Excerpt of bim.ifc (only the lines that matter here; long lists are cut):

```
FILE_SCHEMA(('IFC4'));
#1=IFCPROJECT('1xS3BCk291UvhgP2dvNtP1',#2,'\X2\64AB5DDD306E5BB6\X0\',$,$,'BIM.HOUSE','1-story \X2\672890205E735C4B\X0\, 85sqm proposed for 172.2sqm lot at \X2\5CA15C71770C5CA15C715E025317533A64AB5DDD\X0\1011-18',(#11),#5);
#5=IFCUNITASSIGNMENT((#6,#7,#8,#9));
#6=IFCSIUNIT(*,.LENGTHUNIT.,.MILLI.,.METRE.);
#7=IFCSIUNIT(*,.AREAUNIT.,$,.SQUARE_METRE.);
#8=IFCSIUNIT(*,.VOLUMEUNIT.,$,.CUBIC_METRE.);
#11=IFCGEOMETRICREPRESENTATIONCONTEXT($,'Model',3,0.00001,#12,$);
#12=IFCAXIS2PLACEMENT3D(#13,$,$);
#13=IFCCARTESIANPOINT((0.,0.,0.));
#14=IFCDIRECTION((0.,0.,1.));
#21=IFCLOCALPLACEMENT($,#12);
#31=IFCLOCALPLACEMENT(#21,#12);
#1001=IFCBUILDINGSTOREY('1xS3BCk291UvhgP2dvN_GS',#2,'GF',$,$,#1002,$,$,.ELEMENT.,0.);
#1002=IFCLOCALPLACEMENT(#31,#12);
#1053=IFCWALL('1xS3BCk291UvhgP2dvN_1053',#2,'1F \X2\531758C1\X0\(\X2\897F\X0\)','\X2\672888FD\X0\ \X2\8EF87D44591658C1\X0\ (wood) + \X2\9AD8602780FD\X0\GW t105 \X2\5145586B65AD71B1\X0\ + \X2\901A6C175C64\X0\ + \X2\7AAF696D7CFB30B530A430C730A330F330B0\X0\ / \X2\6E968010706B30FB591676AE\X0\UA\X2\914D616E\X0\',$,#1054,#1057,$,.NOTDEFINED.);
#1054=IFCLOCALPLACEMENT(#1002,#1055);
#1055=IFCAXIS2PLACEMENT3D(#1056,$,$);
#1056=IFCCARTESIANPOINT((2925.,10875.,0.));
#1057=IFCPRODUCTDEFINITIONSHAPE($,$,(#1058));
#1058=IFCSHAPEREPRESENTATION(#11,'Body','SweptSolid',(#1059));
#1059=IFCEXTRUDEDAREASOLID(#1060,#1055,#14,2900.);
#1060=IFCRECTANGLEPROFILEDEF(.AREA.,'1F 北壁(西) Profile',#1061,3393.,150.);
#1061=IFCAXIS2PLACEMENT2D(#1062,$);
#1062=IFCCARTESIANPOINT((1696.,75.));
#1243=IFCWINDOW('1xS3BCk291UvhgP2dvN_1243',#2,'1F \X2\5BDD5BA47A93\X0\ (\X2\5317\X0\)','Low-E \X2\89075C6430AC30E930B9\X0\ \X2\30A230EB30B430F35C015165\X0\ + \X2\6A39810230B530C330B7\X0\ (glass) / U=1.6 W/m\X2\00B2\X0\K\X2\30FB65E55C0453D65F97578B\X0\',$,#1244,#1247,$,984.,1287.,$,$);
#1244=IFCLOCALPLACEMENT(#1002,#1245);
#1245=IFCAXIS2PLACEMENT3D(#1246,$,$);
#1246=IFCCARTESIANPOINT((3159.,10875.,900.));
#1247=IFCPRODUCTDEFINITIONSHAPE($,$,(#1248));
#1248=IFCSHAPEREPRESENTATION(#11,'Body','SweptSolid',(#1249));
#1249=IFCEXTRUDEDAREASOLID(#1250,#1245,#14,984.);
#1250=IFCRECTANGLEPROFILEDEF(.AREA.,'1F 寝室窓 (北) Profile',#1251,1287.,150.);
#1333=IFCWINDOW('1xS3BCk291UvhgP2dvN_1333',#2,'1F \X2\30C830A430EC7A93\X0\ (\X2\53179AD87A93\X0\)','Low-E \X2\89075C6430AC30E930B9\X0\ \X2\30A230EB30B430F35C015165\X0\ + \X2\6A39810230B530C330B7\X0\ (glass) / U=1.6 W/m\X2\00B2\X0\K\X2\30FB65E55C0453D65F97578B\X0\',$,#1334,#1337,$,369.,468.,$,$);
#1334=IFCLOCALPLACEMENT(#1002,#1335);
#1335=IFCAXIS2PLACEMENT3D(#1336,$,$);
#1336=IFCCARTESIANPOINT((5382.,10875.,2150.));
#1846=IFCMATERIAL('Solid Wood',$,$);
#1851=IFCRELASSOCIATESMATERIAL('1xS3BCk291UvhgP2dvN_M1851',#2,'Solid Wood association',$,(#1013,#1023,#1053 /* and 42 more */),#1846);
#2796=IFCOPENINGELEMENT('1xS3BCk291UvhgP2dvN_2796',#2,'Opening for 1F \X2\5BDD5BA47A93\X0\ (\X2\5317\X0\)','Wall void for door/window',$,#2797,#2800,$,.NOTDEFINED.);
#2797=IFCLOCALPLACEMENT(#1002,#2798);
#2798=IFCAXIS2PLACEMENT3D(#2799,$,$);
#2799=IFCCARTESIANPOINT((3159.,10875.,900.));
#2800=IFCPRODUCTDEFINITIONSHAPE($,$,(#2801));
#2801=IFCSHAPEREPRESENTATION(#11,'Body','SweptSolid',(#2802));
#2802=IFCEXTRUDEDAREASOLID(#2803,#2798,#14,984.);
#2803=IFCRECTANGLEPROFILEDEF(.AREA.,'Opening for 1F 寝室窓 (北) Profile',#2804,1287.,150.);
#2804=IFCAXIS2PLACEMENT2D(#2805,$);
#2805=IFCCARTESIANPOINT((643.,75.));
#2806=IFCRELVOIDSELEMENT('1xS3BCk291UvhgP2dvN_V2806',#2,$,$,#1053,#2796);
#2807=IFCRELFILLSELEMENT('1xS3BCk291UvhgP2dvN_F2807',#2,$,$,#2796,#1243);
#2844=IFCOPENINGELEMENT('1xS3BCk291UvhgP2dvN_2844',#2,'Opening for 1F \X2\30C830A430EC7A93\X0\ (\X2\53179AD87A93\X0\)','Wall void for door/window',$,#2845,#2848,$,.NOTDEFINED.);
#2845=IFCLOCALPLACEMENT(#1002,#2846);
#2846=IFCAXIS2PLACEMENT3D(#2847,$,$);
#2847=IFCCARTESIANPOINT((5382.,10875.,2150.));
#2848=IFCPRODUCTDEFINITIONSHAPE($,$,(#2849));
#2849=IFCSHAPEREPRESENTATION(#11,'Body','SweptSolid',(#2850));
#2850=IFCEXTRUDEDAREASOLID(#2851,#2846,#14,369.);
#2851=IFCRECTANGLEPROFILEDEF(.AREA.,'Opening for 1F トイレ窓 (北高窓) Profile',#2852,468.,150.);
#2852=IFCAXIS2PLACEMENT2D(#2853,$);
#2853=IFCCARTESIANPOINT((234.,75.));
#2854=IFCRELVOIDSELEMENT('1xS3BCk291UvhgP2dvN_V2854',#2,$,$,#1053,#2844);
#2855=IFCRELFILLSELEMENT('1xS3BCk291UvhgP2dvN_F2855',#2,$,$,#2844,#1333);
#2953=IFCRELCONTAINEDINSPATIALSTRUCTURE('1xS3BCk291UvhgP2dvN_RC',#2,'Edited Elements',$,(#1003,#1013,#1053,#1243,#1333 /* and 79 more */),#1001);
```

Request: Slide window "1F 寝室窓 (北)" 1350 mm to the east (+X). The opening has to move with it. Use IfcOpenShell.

```python
import ifcopenshell
import ifcopenshell.api.geometry
import ifcopenshell.util.placement
import ifcopenshell.util.unit

model = ifcopenshell.open("bim.ifc")
unit_scale = ifcopenshell.util.unit.calculate_unit_scale(model)

window = model.by_guid("1xS3BCk291UvhgP2dvN_1243")
opening = window.FillsVoids[0].RelatingOpeningElement
wall = opening.VoidsElements[0].RelatingBuildingElement

wall_matrix = ifcopenshell.util.placement.get_local_placement(wall.ObjectPlacement)
shift = wall_matrix[:3, 0] * 1.35 / unit_scale
before = ifcopenshell.util.placement.get_local_placement(window.ObjectPlacement)[:3, 3].copy()

# The window is not placed relative to its opening, so move both.
for product in (opening, window):
    matrix = ifcopenshell.util.placement.get_local_placement(product.ObjectPlacement)
    matrix[:3, 3] += shift
    ifcopenshell.api.geometry.edit_object_placement(model, product=product, matrix=matrix, is_si=False)

after = ifcopenshell.util.placement.get_local_placement(window.ObjectPlacement)[:3, 3]
print("window moved by", (after - before).round(3) + 0.0)

model.write("bim_edited.ifc")
```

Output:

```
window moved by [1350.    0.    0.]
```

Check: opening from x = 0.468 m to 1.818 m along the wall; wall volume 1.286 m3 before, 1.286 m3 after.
